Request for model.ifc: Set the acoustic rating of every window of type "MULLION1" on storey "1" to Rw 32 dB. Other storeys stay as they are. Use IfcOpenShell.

First a look at what the model holds.

```python
import ifcopenshell
import ifcopenshell.util.element

model = ifcopenshell.open("model.ifc")
print(model.schema)
storey = next(s for s in model.by_type("IfcBuildingStorey") if s.Name == "1")
windows = [e for e in ifcopenshell.util.element.get_decomposition(storey) if e.is_a("IfcWindow")]
seen = {}
for e in windows:
    element_type = ifcopenshell.util.element.get_type(e)
    key = (element_type.Name if element_type != e and element_type else None, ifcopenshell.util.element.get_pset(e, "Pset_WindowCommon", "AcousticRating"))
    seen[key] = seen.get(key, 0) + 1
for (name, value), count in sorted(seen.items(), key=str):
    print(count, "x", name, "|", value)
```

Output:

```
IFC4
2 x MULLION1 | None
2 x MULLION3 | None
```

```python
import ifcopenshell
import ifcopenshell.api.pset
import ifcopenshell.util.element

model = ifcopenshell.open("model.ifc")

storey = next(s for s in model.by_type("IfcBuildingStorey") if s.Name == "1")
windows = [e for e in ifcopenshell.util.element.get_decomposition(storey) if e.is_a("IfcWindow")]

count = 0
for e in windows:
    element_type = ifcopenshell.util.element.get_type(e)
    if element_type in (None, e) or element_type.Name != "MULLION1":
        continue
    # add_pset returns the element's existing set when there is one.
    pset = ifcopenshell.api.pset.add_pset(model, product=e, name="Pset_WindowCommon")
    ifcopenshell.api.pset.edit_pset(model, pset=pset, properties={"AcousticRating": "Rw 32 dB"})
    count += 1

print(count, "windows updated")

model.write("model_rev.ifc")
```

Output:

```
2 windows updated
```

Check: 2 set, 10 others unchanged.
